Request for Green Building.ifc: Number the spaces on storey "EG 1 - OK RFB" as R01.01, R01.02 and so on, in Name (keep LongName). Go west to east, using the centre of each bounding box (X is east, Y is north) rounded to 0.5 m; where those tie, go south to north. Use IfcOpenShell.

First a look at what the model holds.

```python
import ifcopenshell
import ifcopenshell.util.element
import ifcopenshell.util.placement

model = ifcopenshell.open("Green Building.ifc")
print(model.schema)
storey = next(s for s in model.by_type("IfcBuildingStorey") if s.Name == "EG 1 - OK RFB")
spaces = [e for e in ifcopenshell.util.element.get_decomposition(storey) if e.is_a("IfcSpace")]
for e in sorted(spaces, key=lambda e: e.id()):
    origin = ifcopenshell.util.placement.get_local_placement(e.ObjectPlacement)[:3, 3]
    print(e.id(), e.Name, e.LongName, origin.round(2) + 0.0, sep=" | ")
```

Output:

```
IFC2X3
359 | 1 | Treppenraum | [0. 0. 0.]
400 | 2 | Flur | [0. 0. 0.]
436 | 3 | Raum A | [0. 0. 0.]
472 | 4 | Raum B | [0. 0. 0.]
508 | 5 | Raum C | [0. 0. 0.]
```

```python
import ifcopenshell
import ifcopenshell.geom
import ifcopenshell.util.element
import ifcopenshell.util.shape

model = ifcopenshell.open("Green Building.ifc")
settings = ifcopenshell.geom.settings()
settings.set("use-world-coords", True)


def centre(element):
    shape = ifcopenshell.geom.create_shape(settings, element)
    return ifcopenshell.util.shape.get_bbox_centroid(shape.geometry)


storey = next(s for s in model.by_type("IfcBuildingStorey") if s.Name == "EG 1 - OK RFB")
spaces = [e for e in ifcopenshell.util.element.get_decomposition(storey) if e.is_a("IfcSpace")]

# Insertion points can sit at a corner or the storey origin, so sort by the geometry (in metres).
centres = {e: centre(e) for e in spaces}
spaces.sort(key=lambda e: (round(centres[e][0] / 0.5), centres[e][1]))

for i, e in enumerate(spaces, start=1):
    number = f"R01.{i:02d}"
    e.Name = number
    print(e.id(), number)

model.write("Green Building-out.ifc")
```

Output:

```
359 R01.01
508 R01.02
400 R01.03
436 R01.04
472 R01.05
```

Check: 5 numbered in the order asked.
